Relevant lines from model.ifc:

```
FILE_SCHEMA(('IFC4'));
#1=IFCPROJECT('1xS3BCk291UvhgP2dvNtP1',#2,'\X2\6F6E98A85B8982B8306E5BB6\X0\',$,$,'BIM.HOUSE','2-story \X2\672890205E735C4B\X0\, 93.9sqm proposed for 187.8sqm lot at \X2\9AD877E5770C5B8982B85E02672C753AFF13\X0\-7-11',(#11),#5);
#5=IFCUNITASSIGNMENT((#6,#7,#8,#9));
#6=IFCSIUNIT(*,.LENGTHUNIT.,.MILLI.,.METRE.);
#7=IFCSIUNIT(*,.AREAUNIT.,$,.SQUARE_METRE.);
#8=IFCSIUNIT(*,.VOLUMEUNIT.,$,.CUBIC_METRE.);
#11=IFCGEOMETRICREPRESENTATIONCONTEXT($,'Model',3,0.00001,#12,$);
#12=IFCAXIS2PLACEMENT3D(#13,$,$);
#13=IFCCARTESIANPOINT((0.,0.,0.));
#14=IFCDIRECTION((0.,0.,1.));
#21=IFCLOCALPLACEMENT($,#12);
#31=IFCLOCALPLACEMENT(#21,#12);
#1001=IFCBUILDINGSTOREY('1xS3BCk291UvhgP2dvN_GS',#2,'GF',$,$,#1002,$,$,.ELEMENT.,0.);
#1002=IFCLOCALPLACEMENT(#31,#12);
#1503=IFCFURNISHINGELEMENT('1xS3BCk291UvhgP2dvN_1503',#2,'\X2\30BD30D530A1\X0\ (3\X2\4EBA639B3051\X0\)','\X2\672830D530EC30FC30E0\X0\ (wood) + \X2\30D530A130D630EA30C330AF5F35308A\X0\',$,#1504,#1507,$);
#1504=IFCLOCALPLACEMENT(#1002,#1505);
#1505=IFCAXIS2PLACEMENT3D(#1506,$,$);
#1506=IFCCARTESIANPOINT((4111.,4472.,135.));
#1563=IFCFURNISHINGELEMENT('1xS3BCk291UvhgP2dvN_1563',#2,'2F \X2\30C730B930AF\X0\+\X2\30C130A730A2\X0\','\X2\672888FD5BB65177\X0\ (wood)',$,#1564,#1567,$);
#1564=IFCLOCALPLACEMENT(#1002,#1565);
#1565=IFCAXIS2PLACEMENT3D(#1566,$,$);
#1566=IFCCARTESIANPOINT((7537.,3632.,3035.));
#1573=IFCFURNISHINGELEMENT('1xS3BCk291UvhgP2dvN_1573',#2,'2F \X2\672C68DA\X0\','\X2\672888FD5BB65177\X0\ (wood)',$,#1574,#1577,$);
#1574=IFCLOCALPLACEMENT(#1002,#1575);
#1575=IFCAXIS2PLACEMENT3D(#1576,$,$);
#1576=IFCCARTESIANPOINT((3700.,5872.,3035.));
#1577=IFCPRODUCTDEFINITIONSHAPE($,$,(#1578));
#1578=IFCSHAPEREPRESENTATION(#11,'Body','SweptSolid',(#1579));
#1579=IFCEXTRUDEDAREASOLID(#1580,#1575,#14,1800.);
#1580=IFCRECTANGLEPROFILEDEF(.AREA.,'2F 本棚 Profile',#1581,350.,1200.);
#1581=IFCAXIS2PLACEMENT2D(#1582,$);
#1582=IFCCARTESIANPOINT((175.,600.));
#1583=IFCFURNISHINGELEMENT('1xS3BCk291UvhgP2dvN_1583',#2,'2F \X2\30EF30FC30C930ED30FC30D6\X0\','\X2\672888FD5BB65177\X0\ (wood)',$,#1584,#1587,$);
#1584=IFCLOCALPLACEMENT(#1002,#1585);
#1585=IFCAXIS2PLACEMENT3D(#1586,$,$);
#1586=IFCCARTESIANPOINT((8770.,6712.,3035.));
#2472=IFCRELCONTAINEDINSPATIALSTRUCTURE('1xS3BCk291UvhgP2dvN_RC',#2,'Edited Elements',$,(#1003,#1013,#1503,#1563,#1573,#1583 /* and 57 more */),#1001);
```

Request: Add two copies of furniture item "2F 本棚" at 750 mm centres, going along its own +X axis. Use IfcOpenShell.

```python
import ifcopenshell
import ifcopenshell.api.geometry
import ifcopenshell.api.root
import ifcopenshell.util.element
import ifcopenshell.util.placement
import ifcopenshell.util.unit

model = ifcopenshell.open("model.ifc")
unit_scale = ifcopenshell.util.unit.calculate_unit_scale(model)


def reuse_history(source, copy):
    """copy_class also copies each property set's owner history, people and application; keep the originals."""
    for rel in copy.IsDefinedBy:
        if rel.is_a("IfcRelDefinesByProperties") and (history := rel.RelatingPropertyDefinition.OwnerHistory):
            rel.RelatingPropertyDefinition.OwnerHistory = source.OwnerHistory
            ifcopenshell.util.element.remove_deep2(model, history)


source = model.by_guid("1xS3BCk291UvhgP2dvN_1573")
base = ifcopenshell.util.placement.get_local_placement(source.ObjectPlacement)
step = base[:3, 0] * 0.75 / unit_scale

for i in range(1, 3):
    copy = ifcopenshell.api.root.copy_class(model, product=source)
    copy.Representation = ifcopenshell.util.element.copy_deep(
        model, source.Representation, exclude=["IfcGeometricRepresentationContext", "IfcRepresentationMap"]
    )
    reuse_history(source, copy)
    matrix = base.copy()
    matrix[:3, 3] += i * step
    print("added at", matrix[:3, 3].round(3) + 0.0)
    ifcopenshell.api.geometry.edit_object_placement(model, product=copy, matrix=matrix, is_si=False)

model.write("model_v2.ifc")
```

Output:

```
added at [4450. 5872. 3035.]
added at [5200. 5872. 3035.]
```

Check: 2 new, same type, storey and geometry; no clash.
